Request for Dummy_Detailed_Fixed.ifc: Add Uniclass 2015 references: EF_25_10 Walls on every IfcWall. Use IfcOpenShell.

First a look at what the model holds.

```python
import ifcopenshell

model = ifcopenshell.open("Dummy_Detailed_Fixed.ifc")
print(model.schema)
print("classifications:", [c.Name for c in model.by_type("IfcClassification")])
for ifc_class in ("IfcDoor", "IfcRoof", "IfcStair", "IfcWall", "IfcWindow"):
    print(ifc_class, len(model.by_type(ifc_class)))
```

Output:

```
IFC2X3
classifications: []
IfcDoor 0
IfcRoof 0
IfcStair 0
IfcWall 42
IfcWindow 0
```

```python
import ifcopenshell
import ifcopenshell.api.classification

model = ifcopenshell.open("Dummy_Detailed_Fixed.ifc")

# IFC2X3 requires Source and Edition and has no link from the project to the system.
system = model.create_entity("IfcClassification", Source="NBS", Edition="2015", Name="Uniclass 2015")

codes = {
    "IfcWall": ("EF_25_10", "Walls"),
}
for ifc_class, (code, name) in codes.items():
    products = model.by_type(ifc_class)
    ifcopenshell.api.classification.add_reference(
        model, products=products, classification=system, identification=code, name=name
    )
    print(code, len(products))

model.write("Dummy_Detailed_Fixed_rev.ifc")
```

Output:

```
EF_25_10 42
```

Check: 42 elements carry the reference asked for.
